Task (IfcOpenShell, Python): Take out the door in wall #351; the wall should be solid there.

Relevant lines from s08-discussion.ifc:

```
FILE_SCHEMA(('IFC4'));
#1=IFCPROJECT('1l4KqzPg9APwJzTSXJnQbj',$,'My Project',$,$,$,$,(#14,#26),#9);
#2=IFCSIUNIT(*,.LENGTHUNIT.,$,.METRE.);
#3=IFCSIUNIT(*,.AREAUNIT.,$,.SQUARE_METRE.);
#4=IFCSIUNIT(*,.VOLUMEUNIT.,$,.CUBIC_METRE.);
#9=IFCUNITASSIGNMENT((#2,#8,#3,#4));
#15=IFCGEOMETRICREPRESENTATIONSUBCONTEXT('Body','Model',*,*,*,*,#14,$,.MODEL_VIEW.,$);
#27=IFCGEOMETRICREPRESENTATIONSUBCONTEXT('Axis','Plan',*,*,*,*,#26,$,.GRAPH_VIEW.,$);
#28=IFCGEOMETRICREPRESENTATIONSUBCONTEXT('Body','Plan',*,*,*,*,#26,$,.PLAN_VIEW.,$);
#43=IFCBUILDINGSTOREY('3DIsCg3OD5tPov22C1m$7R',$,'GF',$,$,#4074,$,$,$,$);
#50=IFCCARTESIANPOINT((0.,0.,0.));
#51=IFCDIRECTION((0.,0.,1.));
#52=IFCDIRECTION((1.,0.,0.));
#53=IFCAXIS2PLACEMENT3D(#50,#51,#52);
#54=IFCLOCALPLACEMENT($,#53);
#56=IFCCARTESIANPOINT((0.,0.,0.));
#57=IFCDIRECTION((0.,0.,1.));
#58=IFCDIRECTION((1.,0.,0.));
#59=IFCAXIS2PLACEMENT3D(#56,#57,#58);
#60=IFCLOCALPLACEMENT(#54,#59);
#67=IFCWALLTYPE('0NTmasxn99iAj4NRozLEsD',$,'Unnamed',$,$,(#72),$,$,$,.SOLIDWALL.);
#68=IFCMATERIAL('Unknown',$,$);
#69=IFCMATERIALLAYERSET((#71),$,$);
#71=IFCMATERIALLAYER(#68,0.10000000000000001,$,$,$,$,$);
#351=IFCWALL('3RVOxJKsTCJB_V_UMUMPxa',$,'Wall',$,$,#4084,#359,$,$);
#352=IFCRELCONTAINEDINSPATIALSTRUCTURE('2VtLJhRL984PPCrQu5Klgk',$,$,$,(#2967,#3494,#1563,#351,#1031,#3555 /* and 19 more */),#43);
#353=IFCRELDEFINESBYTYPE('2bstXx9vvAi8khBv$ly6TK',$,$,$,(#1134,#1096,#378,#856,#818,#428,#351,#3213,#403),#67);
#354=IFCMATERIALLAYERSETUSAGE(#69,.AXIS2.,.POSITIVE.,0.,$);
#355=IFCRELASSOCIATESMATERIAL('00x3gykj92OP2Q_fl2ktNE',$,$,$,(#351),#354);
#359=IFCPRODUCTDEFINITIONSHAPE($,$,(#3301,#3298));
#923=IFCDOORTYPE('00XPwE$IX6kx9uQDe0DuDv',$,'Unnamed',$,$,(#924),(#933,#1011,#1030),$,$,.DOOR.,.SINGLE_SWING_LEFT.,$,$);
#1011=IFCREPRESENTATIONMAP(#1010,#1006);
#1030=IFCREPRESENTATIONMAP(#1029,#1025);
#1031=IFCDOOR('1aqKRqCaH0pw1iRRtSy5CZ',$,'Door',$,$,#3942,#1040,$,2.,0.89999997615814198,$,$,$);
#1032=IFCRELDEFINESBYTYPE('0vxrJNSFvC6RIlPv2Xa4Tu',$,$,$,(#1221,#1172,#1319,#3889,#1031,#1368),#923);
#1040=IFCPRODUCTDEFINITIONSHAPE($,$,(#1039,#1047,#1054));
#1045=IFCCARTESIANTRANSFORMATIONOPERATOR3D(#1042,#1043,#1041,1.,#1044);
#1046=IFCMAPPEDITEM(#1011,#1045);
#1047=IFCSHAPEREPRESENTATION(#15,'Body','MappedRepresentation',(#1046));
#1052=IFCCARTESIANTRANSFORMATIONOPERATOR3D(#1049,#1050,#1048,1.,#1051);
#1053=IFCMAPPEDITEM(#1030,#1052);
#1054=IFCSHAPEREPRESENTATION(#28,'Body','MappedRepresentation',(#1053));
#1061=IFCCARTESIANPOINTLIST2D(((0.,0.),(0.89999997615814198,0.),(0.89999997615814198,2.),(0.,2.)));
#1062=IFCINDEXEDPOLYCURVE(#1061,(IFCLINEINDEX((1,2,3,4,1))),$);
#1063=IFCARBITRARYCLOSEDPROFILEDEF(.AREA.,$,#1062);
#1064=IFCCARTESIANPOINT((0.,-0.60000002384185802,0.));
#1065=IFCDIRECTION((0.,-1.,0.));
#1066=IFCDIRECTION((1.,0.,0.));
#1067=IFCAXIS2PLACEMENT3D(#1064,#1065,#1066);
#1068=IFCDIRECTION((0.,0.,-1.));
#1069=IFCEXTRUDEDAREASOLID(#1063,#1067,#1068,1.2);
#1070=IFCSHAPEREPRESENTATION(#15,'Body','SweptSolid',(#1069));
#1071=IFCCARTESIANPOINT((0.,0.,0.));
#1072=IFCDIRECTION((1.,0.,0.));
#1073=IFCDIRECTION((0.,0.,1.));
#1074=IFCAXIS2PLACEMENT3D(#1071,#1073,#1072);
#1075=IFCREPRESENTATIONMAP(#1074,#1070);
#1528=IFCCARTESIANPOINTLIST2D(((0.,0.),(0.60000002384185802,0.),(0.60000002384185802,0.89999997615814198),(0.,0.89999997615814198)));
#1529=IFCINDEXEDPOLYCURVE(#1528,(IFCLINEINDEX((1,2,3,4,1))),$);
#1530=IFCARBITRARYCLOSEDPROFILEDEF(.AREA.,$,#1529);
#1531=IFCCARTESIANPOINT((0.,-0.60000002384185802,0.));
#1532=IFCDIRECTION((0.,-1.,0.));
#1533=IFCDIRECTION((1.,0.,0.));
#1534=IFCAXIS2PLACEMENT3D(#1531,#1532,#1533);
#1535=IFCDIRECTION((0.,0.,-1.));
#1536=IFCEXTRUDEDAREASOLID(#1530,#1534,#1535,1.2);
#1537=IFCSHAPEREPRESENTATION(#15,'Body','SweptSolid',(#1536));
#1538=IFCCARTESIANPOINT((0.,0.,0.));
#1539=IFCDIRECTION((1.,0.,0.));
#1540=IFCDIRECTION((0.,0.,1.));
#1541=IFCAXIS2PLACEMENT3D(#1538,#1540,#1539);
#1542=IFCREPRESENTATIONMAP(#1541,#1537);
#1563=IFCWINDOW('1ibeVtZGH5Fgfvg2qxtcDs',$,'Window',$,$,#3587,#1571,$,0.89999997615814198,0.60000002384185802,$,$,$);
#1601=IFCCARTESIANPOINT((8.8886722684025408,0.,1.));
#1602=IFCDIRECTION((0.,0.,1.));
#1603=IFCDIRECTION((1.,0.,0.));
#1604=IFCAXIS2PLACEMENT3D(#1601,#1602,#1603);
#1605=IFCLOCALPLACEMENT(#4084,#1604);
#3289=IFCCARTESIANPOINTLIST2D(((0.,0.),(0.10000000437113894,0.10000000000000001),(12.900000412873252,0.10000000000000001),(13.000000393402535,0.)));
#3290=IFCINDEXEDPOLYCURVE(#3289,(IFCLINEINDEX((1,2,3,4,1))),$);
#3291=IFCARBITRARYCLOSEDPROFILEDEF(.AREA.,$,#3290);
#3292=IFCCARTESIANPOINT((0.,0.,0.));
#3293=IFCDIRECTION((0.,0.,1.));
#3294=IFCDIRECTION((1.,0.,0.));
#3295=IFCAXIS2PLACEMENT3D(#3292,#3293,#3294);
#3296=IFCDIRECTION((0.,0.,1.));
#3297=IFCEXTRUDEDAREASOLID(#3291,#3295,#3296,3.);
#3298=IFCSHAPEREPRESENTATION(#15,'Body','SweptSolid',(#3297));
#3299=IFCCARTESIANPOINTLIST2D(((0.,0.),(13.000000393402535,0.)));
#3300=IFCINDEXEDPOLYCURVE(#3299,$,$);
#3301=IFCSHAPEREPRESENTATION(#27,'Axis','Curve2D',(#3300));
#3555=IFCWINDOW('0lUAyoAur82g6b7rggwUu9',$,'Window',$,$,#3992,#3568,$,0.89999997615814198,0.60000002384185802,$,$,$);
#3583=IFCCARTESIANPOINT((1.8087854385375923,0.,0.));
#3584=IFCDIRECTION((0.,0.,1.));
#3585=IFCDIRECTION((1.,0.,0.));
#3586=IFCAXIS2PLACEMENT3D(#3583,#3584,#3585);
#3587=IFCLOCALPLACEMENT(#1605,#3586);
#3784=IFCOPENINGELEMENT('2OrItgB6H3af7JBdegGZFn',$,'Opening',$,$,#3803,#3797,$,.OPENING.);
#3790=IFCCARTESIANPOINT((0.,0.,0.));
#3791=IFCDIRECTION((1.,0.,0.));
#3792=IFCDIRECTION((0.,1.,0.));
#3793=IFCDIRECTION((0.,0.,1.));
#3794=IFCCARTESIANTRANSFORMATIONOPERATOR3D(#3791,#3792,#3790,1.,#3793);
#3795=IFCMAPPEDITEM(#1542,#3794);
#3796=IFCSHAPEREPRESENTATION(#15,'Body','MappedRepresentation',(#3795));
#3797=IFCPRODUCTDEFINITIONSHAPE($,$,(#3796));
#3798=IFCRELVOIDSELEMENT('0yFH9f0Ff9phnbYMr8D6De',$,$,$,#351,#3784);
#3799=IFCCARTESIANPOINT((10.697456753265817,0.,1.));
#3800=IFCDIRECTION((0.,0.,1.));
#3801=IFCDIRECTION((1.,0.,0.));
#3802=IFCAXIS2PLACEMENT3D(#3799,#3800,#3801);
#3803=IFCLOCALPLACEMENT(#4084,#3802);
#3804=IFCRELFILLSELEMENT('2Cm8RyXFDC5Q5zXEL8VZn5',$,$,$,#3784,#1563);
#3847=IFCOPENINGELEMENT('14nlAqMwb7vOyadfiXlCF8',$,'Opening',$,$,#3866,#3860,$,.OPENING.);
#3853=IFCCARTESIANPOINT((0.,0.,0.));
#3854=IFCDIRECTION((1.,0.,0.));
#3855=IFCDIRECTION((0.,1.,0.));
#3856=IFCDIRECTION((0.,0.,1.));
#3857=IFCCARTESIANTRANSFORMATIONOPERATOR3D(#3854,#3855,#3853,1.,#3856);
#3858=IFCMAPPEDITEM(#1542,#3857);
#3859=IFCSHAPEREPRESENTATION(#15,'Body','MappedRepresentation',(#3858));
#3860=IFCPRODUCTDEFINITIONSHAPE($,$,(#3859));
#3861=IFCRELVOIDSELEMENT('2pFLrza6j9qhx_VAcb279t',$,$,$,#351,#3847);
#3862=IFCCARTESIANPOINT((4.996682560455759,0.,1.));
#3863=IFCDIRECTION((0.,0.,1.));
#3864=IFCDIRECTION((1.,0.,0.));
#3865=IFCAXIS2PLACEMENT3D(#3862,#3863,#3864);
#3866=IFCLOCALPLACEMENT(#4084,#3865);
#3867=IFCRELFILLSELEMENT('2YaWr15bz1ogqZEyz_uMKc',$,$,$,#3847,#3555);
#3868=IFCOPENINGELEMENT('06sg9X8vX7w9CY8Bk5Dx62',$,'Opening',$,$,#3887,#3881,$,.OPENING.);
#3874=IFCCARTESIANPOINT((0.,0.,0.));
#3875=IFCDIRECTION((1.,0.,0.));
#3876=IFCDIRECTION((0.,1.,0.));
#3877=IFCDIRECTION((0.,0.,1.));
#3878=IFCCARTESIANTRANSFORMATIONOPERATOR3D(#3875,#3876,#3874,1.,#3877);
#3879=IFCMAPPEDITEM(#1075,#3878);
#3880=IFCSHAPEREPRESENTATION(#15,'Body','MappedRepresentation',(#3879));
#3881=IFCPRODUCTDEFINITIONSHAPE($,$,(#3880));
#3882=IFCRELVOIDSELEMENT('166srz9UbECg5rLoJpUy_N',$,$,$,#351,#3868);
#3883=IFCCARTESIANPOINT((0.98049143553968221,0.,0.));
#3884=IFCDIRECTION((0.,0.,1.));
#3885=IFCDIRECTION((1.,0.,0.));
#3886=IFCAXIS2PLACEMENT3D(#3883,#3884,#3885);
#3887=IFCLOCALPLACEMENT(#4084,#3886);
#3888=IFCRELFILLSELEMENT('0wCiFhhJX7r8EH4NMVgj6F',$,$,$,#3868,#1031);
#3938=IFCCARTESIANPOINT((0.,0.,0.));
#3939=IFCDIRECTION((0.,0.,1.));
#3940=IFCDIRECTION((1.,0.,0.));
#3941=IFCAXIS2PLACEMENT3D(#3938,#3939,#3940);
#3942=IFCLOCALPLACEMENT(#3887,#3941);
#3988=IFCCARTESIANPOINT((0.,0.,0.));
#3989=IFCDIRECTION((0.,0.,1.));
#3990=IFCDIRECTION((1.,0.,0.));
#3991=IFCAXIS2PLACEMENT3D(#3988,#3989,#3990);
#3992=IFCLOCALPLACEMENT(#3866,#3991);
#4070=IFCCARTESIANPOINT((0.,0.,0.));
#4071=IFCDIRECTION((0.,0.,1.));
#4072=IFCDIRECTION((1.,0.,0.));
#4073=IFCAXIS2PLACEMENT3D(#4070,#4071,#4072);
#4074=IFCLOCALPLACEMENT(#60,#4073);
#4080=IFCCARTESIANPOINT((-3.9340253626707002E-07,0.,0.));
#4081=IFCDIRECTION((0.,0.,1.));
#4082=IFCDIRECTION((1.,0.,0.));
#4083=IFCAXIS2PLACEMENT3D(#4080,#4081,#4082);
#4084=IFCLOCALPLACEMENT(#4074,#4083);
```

```python
import ifcopenshell
import ifcopenshell.api.feature
import ifcopenshell.api.root
import ifcopenshell.geom
import ifcopenshell.util.shape

model = ifcopenshell.open("s08-discussion.ifc")
settings = ifcopenshell.geom.settings()


def volume(element):
    """Net volume in cubic metres, openings subtracted."""
    shape = ifcopenshell.geom.create_shape(settings, element)
    return ifcopenshell.util.shape.get_volume(shape.geometry)


door = model.by_guid("1aqKRqCaH0pw1iRRtSy5CZ")
opening = door.FillsVoids[0].RelatingOpeningElement
wall = opening.VoidsElements[0].RelatingBuildingElement
before = volume(wall)

ifcopenshell.api.root.remove_product(model, product=door)
ifcopenshell.api.feature.remove_feature(model, feature=opening)

after = volume(wall)

print(f"wall volume {before:.3f} -> {after:.3f} m3")

model.write("s08-discussion_v2.ifc")
```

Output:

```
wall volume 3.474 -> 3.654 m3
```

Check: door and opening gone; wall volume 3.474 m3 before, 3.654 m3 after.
